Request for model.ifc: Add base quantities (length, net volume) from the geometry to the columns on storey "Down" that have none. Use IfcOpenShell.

First a look at what the model holds.

```python
import ifcopenshell
import ifcopenshell.util.element
import ifcopenshell.util.unit

model = ifcopenshell.open("model.ifc")
print(model.schema)
for unit_type in ("LENGTHUNIT", "AREAUNIT", "VOLUMEUNIT"):
    print(unit_type, ifcopenshell.util.unit.calculate_unit_scale(model, unit_type))
storey = next(s for s in model.by_type("IfcBuildingStorey") if s.Name == "Down")
columns = [e for e in ifcopenshell.util.element.get_decomposition(storey) if e.is_a("IfcColumn")]
for e in sorted(columns, key=lambda e: e.id()):
    print(e.id(), e.is_a(), e.Name, list(ifcopenshell.util.element.get_psets(e, qtos_only=True)), sep=" | ")
```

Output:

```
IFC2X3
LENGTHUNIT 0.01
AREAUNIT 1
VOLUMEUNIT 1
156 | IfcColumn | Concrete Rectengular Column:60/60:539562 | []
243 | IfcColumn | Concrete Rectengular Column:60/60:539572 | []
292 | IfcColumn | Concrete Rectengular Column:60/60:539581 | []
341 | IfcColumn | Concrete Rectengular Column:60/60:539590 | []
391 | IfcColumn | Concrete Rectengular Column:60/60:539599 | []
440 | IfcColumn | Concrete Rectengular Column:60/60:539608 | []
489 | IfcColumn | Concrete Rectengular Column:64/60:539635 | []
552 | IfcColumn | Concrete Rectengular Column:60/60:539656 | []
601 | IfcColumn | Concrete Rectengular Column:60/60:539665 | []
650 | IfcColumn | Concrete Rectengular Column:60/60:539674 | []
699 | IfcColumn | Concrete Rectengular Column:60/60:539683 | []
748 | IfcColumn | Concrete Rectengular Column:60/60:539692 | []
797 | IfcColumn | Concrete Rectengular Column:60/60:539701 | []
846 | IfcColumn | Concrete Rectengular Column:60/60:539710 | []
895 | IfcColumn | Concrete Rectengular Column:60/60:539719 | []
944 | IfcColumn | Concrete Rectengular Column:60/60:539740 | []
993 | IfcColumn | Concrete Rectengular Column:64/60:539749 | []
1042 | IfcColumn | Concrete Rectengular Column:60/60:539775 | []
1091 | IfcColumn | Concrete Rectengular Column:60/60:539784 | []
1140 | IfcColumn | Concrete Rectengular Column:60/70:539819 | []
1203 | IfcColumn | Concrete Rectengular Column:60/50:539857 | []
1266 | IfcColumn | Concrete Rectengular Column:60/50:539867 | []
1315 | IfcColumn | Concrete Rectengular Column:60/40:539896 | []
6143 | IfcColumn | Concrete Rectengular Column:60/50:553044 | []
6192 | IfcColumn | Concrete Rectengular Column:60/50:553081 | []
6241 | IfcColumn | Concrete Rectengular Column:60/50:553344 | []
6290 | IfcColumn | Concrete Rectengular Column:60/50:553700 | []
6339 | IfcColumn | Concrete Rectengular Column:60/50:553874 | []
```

```python
import ifcopenshell
import ifcopenshell.api.pset
import ifcopenshell.geom
import ifcopenshell.util.element
import ifcopenshell.util.shape
import ifcopenshell.util.unit

model = ifcopenshell.open("model.ifc")
unit_scale = ifcopenshell.util.unit.calculate_unit_scale(model)
volume_scale = ifcopenshell.util.unit.calculate_unit_scale(model, "VOLUMEUNIT")
settings = ifcopenshell.geom.settings()

storey = next(s for s in model.by_type("IfcBuildingStorey") if s.Name == "Down")
columns = [e for e in ifcopenshell.util.element.get_decomposition(storey) if e.is_a("IfcColumn")]

for e in sorted(columns, key=lambda e: e.id()):
    if ifcopenshell.util.element.get_psets(e, qtos_only=True, should_inherit=False):
        continue
    # Geometry comes back in metres, in the element's own axes.
    shape = ifcopenshell.geom.create_shape(settings, e)
    values = {
        "Length": ifcopenshell.util.shape.get_z(shape.geometry) / unit_scale,
        "NetVolume": ifcopenshell.util.shape.get_volume(shape.geometry) / volume_scale,
    }
    qto = ifcopenshell.api.pset.add_qto(model, product=e, name="BaseQuantities")
    ifcopenshell.api.pset.edit_qto(model, qto=qto, properties=values)
    print(e.id(), {k: round(v, 3) for k, v in values.items()})

model.write("model_updated.ifc")
```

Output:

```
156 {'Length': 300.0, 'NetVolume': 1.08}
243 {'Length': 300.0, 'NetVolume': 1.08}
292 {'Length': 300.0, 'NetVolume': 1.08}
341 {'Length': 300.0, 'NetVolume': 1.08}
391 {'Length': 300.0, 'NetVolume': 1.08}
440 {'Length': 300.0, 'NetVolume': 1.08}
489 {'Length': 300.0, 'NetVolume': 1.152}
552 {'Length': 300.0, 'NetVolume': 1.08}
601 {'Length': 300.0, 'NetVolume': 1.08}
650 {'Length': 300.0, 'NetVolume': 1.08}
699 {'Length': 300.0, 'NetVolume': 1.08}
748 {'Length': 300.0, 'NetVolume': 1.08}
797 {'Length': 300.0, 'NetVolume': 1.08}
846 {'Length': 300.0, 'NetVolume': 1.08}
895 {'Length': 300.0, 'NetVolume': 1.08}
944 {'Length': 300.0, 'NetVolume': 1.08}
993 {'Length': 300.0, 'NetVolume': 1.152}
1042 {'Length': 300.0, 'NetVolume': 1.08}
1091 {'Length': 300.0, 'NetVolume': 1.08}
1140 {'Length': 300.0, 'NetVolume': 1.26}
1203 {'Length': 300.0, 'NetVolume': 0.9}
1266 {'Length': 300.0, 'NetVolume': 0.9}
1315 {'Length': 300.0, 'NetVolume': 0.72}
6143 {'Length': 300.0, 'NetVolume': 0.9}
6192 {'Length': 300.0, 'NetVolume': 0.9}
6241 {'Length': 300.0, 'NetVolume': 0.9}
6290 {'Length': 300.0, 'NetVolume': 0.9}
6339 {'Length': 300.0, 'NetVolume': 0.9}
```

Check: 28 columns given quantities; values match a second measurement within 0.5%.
